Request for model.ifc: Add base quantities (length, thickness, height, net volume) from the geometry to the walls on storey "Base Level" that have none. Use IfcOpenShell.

First a look at what the model holds.

```python
import ifcopenshell
import ifcopenshell.util.element
import ifcopenshell.util.unit

model = ifcopenshell.open("model.ifc")
print(model.schema)
for unit_type in ("LENGTHUNIT", "AREAUNIT", "VOLUMEUNIT"):
    print(unit_type, ifcopenshell.util.unit.calculate_unit_scale(model, unit_type))
storey = next(s for s in model.by_type("IfcBuildingStorey") if s.Name == "Base Level")
walls = [e for e in ifcopenshell.util.element.get_decomposition(storey) if e.is_a("IfcWall")]
for e in sorted(walls, key=lambda e: e.id()):
    print(e.id(), e.is_a(), e.Name, list(ifcopenshell.util.element.get_psets(e, qtos_only=True)), sep=" | ")
```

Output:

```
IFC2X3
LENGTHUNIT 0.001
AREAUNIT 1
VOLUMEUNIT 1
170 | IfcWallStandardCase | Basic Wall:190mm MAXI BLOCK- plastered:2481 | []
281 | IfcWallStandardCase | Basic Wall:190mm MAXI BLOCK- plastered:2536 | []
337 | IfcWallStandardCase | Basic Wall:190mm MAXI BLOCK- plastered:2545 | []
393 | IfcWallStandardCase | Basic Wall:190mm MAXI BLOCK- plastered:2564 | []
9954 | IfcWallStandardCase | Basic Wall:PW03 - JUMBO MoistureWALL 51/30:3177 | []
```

```python
import ifcopenshell
import ifcopenshell.api.pset
import ifcopenshell.geom
import ifcopenshell.util.element
import ifcopenshell.util.shape
import ifcopenshell.util.unit

model = ifcopenshell.open("model.ifc")
unit_scale = ifcopenshell.util.unit.calculate_unit_scale(model)
volume_scale = ifcopenshell.util.unit.calculate_unit_scale(model, "VOLUMEUNIT")
settings = ifcopenshell.geom.settings()

storey = next(s for s in model.by_type("IfcBuildingStorey") if s.Name == "Base Level")
walls = [e for e in ifcopenshell.util.element.get_decomposition(storey) if e.is_a("IfcWall")]

for e in sorted(walls, key=lambda e: e.id()):
    if ifcopenshell.util.element.get_psets(e, qtos_only=True, should_inherit=False):
        continue
    # Geometry comes back in metres, in the element's own axes.
    shape = ifcopenshell.geom.create_shape(settings, e)
    values = {
        "Length": ifcopenshell.util.shape.get_x(shape.geometry) / unit_scale,
        "Width": ifcopenshell.util.shape.get_y(shape.geometry) / unit_scale,
        "Height": ifcopenshell.util.shape.get_z(shape.geometry) / unit_scale,
        "NetVolume": ifcopenshell.util.shape.get_volume(shape.geometry) / volume_scale,
    }
    qto = ifcopenshell.api.pset.add_qto(model, product=e, name="BaseQuantities")
    ifcopenshell.api.pset.edit_qto(model, qto=qto, properties=values)
    print(e.id(), {k: round(v, 3) for k, v in values.items()})

model.write("model_v2.ifc")
```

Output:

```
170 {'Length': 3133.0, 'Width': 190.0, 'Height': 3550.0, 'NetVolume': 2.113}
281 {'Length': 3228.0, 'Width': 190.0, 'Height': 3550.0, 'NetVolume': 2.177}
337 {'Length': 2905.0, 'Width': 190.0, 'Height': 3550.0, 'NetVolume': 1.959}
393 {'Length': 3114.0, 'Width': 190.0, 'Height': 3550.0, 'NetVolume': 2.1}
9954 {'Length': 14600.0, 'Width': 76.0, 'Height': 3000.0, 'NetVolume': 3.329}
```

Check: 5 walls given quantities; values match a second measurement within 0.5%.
